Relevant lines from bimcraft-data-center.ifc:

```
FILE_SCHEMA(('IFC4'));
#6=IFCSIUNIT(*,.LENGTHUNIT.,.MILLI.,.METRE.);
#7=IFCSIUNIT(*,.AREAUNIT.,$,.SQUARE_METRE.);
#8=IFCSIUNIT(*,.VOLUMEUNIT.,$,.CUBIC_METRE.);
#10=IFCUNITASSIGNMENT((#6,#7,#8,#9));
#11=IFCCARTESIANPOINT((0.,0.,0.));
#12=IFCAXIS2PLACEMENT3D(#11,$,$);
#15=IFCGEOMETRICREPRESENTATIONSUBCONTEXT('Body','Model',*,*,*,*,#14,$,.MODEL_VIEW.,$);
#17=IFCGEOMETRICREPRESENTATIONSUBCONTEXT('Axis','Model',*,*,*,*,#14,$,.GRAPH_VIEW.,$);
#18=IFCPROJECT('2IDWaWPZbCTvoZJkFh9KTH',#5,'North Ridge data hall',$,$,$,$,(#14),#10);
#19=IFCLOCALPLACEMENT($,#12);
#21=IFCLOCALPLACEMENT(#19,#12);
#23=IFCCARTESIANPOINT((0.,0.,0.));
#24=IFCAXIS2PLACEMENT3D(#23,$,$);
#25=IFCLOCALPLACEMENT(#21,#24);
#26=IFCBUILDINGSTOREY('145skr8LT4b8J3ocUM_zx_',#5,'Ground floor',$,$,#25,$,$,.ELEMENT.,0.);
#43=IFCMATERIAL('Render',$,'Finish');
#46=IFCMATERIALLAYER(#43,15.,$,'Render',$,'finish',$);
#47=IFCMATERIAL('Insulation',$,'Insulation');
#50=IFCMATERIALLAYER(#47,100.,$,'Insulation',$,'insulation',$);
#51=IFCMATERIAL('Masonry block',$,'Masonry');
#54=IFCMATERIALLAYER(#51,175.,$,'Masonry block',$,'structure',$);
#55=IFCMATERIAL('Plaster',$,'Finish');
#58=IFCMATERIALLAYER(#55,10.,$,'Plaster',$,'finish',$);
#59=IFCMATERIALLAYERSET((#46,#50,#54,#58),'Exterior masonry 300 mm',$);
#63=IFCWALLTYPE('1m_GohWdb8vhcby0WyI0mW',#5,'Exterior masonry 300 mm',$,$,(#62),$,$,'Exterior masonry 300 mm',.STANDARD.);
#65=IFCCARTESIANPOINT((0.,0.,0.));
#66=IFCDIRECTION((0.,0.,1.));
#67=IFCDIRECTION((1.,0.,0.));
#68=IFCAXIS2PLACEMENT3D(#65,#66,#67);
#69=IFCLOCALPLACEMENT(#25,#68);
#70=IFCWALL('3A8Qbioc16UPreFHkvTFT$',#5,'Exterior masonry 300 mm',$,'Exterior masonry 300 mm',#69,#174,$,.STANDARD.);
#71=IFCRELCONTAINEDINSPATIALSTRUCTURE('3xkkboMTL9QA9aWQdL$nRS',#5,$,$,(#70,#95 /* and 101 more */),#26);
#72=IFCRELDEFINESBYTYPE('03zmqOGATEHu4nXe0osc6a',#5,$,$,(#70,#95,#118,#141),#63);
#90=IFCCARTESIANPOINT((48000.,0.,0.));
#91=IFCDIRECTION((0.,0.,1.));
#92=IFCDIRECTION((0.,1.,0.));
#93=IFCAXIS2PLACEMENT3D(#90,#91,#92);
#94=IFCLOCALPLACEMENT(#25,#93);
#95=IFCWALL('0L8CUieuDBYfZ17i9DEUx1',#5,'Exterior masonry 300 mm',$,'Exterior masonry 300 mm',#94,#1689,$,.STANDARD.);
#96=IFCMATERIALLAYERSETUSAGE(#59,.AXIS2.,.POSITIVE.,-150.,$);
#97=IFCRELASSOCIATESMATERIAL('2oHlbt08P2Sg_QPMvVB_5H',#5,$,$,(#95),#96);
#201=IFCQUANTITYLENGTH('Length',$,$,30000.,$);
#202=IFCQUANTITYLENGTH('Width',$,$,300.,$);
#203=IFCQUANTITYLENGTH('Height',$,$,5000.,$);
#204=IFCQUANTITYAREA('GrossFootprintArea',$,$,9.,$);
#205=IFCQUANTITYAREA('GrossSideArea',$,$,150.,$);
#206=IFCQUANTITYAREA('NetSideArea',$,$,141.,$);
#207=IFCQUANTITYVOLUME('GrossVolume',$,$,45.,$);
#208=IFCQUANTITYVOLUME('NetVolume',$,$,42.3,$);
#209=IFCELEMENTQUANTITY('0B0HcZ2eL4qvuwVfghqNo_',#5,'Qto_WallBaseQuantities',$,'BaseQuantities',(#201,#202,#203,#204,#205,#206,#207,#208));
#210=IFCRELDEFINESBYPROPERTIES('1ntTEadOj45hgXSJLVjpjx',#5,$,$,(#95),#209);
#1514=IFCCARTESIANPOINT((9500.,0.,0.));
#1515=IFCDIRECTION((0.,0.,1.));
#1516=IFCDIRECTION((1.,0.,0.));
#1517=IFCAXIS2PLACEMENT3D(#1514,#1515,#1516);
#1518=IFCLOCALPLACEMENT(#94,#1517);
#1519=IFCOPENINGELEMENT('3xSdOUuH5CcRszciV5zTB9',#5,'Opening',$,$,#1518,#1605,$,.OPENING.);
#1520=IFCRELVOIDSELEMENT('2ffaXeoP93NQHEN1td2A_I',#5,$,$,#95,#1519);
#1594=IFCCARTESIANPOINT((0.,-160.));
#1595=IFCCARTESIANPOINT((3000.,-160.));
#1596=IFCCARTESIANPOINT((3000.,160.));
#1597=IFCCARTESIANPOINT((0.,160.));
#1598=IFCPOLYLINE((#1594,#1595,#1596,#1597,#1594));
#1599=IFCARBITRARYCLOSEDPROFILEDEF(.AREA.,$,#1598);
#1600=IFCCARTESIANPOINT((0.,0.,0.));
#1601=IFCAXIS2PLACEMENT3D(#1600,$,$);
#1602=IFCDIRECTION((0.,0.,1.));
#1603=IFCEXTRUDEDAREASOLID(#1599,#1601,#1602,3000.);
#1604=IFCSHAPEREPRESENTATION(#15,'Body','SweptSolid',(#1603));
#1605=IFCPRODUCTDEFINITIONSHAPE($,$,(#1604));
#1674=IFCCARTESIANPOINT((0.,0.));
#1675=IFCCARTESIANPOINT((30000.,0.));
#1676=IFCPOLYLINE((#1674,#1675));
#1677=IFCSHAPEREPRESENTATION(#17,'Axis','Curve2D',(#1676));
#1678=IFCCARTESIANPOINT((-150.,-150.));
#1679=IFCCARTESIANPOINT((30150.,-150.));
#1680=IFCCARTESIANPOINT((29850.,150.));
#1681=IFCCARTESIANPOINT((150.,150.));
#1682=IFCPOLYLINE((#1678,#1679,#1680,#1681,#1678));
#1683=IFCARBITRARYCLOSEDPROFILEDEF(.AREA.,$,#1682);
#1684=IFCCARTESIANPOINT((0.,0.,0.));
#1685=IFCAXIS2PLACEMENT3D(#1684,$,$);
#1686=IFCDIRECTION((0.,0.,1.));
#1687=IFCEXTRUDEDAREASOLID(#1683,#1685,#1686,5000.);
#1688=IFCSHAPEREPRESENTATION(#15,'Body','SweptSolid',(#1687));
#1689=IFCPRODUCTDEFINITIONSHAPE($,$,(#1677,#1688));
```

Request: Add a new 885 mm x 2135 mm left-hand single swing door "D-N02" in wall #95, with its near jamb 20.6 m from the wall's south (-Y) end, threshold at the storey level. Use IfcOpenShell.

```python
import numpy as np
import ifcopenshell
import ifcopenshell.api.feature
import ifcopenshell.api.geometry
import ifcopenshell.api.pset
import ifcopenshell.api.root
import ifcopenshell.api.spatial
import ifcopenshell.geom
import ifcopenshell.util.element
import ifcopenshell.util.placement
import ifcopenshell.util.representation
import ifcopenshell.util.shape
import ifcopenshell.util.unit

model = ifcopenshell.open("bimcraft-data-center.ifc")
unit_scale = ifcopenshell.util.unit.calculate_unit_scale(model)
area_scale = ifcopenshell.util.unit.calculate_unit_scale(model, "AREAUNIT")
volume_scale = ifcopenshell.util.unit.calculate_unit_scale(model, "VOLUMEUNIT")
settings = ifcopenshell.geom.settings()


def volume(element):
    """Net volume in cubic metres, openings subtracted."""
    shape = ifcopenshell.geom.create_shape(settings, element)
    return ifcopenshell.util.shape.get_volume(shape.geometry)


wall = model.by_guid("0L8CUieuDBYfZ17i9DEUx1")
storey = ifcopenshell.util.element.get_container(wall, ifc_class="IfcBuildingStorey")
context = ifcopenshell.util.representation.get_context(model, "Model", "Body", "MODEL_VIEW")
before = volume(wall)

width, height, from_end, sill = 0.885, 2.135, 20.6, 0.0  # metres

# The wall runs along its own X axis, and the end named is its -X end.
wall_shape = ifcopenshell.geom.create_shape(settings, wall)
x, y, z = ifcopenshell.util.shape.get_vertices(wall_shape.geometry).T
start = x.min() + from_end
face, thickness = float(y.min()), float(y.max() - y.min())
wall_matrix = ifcopenshell.util.placement.get_local_placement(wall.ObjectPlacement)
level = ifcopenshell.util.placement.get_local_placement(storey.ObjectPlacement)[2, 3]


def in_wall(x, y):
    """Placement at x, y metres in the wall's axes, at sill height."""
    matrix = wall_matrix.copy()
    matrix[:, 3] = wall_matrix @ np.array([x / unit_scale, y / unit_scale, 0.0, 1.0])
    matrix[2, 3] = level + sill / unit_scale
    return matrix


# Opening: a box that overshoots both wall faces by 50 mm.
opening = ifcopenshell.api.root.create_entity(model, ifc_class="IfcOpeningElement", predefined_type="OPENING")
box = ifcopenshell.api.geometry.add_wall_representation(
    model, context=context, length=width, height=height, thickness=thickness + 0.1
)
ifcopenshell.api.geometry.assign_representation(model, product=opening, representation=box)
ifcopenshell.api.geometry.edit_object_placement(model, product=opening, matrix=in_wall(start, face - 0.05), is_si=False)
ifcopenshell.api.feature.add_feature(model, feature=opening, element=wall)

door = ifcopenshell.api.root.create_entity(model, ifc_class="IfcDoor", name="D-N02", predefined_type="DOOR")
door.OverallWidth, door.OverallHeight = width / unit_scale, height / unit_scale
door.OperationType = "SINGLE_SWING_LEFT"
body = ifcopenshell.api.geometry.add_door_representation(
    model,
    context=context,
    overall_width=door.OverallWidth,
    overall_height=door.OverallHeight,
    operation_type="SINGLE_SWING_LEFT",
    lining_properties={"LiningDepth": thickness / unit_scale, "ThresholdDepth": thickness / unit_scale},
)
ifcopenshell.api.geometry.assign_representation(model, product=door, representation=body)
ifcopenshell.api.spatial.assign_container(model, products=[door], relating_structure=storey)
ifcopenshell.api.feature.add_filling(model, opening=opening, element=door)

# The lining spans the wall, so the door starts at the wall face.
ifcopenshell.api.geometry.edit_object_placement(model, product=door, matrix=in_wall(start, face), is_si=False)

after = volume(wall)

# Update the wall's stored quantities.
qto = model.by_id(ifcopenshell.util.element.get_pset(wall, "Qto_WallBaseQuantities", should_inherit=False)["id"])
ifcopenshell.api.pset.edit_qto(model, qto=qto, properties={
    "NetSideArea": after / thickness / area_scale,
    "NetVolume": after / volume_scale,
})

print(f"wall volume {before:.3f} -> {after:.3f} m3")

model.write("bimcraft-data-center-out.ifc")
```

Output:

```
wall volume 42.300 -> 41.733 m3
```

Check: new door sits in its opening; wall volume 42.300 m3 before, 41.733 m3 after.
